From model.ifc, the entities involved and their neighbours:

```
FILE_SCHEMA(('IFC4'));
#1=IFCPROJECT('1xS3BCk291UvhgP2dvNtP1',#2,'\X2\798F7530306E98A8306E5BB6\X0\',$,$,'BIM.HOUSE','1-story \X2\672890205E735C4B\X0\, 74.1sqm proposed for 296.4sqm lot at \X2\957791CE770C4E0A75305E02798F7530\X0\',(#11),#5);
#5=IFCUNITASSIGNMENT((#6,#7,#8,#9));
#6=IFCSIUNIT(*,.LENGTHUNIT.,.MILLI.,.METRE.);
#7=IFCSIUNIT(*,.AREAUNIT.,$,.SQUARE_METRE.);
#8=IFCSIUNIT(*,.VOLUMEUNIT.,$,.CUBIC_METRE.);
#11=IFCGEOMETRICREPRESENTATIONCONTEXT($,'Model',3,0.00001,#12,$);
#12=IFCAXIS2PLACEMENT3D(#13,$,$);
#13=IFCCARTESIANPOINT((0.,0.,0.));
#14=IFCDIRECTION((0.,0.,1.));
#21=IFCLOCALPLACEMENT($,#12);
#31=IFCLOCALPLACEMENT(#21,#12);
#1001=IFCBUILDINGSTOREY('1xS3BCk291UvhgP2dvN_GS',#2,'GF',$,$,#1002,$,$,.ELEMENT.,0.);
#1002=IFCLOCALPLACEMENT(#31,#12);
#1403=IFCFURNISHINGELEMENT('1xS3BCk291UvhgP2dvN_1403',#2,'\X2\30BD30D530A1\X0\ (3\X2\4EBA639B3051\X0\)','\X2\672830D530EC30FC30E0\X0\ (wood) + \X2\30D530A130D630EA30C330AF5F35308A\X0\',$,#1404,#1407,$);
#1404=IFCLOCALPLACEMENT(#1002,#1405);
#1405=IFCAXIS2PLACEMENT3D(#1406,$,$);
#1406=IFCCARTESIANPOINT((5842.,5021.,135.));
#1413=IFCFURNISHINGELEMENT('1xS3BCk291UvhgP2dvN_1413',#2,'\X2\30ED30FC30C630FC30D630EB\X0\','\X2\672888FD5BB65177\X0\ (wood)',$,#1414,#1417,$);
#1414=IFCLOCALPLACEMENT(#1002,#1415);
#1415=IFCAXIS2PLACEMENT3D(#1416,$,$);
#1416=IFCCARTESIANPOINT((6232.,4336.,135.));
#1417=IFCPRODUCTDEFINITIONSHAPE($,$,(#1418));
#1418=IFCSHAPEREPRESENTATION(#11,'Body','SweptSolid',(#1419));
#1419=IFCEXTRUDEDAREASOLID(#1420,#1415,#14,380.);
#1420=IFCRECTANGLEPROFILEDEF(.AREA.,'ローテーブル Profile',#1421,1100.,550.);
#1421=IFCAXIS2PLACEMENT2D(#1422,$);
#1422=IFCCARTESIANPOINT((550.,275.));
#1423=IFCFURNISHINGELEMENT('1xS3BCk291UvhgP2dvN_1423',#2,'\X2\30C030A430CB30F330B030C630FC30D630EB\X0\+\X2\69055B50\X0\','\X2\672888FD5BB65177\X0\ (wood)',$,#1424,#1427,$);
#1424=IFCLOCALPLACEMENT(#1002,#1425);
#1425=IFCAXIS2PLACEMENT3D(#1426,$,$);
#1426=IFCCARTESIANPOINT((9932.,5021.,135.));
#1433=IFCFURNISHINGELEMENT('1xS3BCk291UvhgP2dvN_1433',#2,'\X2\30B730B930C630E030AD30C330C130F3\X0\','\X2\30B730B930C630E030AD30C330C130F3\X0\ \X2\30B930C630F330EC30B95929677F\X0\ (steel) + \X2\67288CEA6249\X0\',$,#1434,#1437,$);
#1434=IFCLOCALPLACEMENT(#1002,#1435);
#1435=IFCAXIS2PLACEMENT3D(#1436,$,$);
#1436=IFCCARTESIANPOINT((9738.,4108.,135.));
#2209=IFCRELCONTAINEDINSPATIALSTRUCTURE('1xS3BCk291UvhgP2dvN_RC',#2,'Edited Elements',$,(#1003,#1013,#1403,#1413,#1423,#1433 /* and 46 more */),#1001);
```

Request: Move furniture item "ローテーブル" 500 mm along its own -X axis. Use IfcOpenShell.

```python
import ifcopenshell
import ifcopenshell.api.geometry
import ifcopenshell.util.placement

model = ifcopenshell.open("model.ifc")

item = model.by_id(1413)
matrix = ifcopenshell.util.placement.get_local_placement(item.ObjectPlacement)
matrix[:3, 3] -= matrix[:3, 0] * 500.0
ifcopenshell.api.geometry.edit_object_placement(model, product=item, matrix=matrix, is_si=False)

print(ifcopenshell.util.placement.get_local_placement(item.ObjectPlacement).round(3) + 0.0)

model.write("model_rev.ifc")
```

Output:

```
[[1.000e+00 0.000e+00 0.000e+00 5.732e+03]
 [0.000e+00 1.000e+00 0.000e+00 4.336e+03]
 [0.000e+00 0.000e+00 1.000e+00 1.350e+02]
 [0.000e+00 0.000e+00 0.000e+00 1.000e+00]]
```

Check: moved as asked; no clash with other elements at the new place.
